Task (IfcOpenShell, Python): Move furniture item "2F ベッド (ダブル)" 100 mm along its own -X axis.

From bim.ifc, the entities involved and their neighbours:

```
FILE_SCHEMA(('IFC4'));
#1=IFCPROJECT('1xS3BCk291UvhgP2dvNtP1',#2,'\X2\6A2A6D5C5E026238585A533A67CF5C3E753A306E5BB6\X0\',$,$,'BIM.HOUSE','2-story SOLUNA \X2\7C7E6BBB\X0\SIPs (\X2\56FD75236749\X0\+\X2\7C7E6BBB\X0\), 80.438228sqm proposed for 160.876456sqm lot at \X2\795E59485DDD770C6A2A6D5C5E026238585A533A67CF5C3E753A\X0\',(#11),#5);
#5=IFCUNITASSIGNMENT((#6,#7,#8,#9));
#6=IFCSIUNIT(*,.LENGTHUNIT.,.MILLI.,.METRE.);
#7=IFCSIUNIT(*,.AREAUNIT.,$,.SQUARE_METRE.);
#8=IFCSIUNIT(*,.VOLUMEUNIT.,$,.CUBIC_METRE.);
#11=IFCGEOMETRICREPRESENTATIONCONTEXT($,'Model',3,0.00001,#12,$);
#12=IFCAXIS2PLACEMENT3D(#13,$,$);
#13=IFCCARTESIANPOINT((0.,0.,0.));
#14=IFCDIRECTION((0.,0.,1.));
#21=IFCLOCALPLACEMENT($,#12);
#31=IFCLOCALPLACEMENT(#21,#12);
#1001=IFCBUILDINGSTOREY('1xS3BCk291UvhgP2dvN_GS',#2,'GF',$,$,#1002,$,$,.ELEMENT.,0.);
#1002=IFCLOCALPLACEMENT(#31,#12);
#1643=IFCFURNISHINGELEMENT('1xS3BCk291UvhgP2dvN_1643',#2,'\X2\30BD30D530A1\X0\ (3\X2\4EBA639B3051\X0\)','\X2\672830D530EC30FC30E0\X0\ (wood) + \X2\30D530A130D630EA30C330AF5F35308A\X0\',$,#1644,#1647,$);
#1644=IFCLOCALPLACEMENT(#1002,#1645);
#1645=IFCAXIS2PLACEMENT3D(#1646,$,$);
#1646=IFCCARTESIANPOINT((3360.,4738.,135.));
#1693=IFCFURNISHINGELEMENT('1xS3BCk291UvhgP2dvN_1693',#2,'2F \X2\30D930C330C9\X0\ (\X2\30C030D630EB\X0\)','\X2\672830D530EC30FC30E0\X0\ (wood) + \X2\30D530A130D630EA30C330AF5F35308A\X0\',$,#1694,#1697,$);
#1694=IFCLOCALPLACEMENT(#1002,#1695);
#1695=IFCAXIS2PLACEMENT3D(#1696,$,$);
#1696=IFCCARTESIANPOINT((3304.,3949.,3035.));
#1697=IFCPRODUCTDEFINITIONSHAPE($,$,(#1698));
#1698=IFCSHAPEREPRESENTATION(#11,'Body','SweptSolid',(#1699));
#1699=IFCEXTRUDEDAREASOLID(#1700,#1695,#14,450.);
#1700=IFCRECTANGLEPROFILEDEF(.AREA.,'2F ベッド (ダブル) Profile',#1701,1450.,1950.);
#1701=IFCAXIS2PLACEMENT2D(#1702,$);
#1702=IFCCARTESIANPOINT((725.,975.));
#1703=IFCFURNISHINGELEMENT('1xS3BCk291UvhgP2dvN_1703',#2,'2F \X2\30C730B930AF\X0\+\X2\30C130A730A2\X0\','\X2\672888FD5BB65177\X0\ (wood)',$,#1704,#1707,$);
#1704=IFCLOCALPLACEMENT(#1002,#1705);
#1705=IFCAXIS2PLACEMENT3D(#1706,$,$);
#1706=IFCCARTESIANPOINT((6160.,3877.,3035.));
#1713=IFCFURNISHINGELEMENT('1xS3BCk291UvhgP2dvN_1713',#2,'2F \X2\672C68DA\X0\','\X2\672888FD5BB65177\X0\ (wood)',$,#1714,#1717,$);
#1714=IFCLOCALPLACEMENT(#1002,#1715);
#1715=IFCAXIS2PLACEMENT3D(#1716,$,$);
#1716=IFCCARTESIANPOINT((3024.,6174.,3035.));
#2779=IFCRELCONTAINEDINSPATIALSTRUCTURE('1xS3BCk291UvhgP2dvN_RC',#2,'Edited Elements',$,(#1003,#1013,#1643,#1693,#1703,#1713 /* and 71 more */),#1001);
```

```python
import ifcopenshell
import ifcopenshell.api.geometry
import ifcopenshell.util.placement

model = ifcopenshell.open("bim.ifc")

item = model.by_guid("1xS3BCk291UvhgP2dvN_1693")
matrix = ifcopenshell.util.placement.get_local_placement(item.ObjectPlacement)
matrix[:3, 3] -= matrix[:3, 0] * 100.0
ifcopenshell.api.geometry.edit_object_placement(model, product=item, matrix=matrix, is_si=False)

print(ifcopenshell.util.placement.get_local_placement(item.ObjectPlacement).round(3) + 0.0)

model.write("bim_edited.ifc")
```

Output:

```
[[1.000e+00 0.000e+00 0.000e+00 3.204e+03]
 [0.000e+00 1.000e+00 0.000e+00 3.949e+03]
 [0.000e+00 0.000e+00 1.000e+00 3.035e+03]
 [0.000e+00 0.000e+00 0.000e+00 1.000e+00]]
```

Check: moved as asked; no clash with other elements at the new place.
